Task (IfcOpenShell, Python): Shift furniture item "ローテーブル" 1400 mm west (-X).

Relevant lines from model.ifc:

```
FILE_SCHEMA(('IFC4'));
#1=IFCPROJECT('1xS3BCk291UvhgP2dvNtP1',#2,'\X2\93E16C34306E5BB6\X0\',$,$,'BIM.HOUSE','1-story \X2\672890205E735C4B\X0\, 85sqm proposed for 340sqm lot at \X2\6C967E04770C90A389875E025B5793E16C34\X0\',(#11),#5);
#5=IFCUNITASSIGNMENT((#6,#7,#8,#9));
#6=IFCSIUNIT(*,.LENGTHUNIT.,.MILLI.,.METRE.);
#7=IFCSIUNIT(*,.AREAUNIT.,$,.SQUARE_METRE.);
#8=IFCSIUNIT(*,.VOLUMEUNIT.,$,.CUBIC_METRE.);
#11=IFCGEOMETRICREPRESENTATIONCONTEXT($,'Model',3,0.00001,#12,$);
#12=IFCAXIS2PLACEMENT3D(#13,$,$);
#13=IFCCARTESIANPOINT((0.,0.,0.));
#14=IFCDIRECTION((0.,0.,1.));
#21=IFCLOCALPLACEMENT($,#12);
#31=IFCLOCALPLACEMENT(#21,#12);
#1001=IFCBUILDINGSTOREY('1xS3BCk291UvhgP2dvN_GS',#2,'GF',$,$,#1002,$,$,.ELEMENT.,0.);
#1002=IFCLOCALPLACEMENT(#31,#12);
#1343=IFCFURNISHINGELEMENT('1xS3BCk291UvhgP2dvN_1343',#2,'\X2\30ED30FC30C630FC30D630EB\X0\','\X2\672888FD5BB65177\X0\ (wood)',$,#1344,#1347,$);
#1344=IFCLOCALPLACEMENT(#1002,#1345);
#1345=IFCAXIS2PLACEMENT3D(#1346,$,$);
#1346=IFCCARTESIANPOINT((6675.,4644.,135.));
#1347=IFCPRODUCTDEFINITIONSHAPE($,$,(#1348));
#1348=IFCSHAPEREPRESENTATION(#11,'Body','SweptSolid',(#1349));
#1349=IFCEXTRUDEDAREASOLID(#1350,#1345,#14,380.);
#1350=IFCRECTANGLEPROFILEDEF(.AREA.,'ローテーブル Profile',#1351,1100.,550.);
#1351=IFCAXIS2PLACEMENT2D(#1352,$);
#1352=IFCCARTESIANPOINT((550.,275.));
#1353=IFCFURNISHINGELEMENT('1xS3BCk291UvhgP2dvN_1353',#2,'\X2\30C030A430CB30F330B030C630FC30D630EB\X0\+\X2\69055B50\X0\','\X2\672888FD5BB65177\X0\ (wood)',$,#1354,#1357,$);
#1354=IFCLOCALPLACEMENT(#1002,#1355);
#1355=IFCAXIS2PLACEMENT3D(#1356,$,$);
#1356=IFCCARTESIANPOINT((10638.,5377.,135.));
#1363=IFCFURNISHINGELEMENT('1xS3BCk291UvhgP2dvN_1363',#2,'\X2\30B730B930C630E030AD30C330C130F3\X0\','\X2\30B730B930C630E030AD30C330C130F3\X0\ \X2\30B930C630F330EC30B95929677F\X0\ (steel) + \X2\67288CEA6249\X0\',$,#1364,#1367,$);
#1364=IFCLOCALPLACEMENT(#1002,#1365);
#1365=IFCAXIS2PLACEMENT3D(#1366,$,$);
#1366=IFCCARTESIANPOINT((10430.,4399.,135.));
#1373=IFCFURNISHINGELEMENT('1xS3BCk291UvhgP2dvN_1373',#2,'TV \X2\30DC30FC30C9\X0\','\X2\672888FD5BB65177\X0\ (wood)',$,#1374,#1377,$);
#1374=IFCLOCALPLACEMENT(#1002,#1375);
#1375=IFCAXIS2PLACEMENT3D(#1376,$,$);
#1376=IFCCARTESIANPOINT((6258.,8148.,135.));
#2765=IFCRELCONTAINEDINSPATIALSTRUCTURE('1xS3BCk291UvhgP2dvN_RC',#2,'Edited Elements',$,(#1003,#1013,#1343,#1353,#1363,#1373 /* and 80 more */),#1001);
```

```python
import ifcopenshell
import ifcopenshell.api.geometry
import ifcopenshell.util.placement
import ifcopenshell.util.unit

model = ifcopenshell.open("model.ifc")
unit_scale = ifcopenshell.util.unit.calculate_unit_scale(model)

item = model.by_guid("1xS3BCk291UvhgP2dvN_1343")
matrix = ifcopenshell.util.placement.get_local_placement(item.ObjectPlacement)
matrix[0, 3] -= 1.4 / unit_scale
ifcopenshell.api.geometry.edit_object_placement(model, product=item, matrix=matrix, is_si=False)

print(ifcopenshell.util.placement.get_local_placement(item.ObjectPlacement).round(3) + 0.0)

model.write("model_edited.ifc")
```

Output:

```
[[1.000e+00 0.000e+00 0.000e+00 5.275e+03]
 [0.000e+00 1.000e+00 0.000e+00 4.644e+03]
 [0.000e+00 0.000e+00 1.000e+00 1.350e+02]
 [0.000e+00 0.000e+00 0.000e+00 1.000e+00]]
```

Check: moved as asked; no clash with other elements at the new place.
